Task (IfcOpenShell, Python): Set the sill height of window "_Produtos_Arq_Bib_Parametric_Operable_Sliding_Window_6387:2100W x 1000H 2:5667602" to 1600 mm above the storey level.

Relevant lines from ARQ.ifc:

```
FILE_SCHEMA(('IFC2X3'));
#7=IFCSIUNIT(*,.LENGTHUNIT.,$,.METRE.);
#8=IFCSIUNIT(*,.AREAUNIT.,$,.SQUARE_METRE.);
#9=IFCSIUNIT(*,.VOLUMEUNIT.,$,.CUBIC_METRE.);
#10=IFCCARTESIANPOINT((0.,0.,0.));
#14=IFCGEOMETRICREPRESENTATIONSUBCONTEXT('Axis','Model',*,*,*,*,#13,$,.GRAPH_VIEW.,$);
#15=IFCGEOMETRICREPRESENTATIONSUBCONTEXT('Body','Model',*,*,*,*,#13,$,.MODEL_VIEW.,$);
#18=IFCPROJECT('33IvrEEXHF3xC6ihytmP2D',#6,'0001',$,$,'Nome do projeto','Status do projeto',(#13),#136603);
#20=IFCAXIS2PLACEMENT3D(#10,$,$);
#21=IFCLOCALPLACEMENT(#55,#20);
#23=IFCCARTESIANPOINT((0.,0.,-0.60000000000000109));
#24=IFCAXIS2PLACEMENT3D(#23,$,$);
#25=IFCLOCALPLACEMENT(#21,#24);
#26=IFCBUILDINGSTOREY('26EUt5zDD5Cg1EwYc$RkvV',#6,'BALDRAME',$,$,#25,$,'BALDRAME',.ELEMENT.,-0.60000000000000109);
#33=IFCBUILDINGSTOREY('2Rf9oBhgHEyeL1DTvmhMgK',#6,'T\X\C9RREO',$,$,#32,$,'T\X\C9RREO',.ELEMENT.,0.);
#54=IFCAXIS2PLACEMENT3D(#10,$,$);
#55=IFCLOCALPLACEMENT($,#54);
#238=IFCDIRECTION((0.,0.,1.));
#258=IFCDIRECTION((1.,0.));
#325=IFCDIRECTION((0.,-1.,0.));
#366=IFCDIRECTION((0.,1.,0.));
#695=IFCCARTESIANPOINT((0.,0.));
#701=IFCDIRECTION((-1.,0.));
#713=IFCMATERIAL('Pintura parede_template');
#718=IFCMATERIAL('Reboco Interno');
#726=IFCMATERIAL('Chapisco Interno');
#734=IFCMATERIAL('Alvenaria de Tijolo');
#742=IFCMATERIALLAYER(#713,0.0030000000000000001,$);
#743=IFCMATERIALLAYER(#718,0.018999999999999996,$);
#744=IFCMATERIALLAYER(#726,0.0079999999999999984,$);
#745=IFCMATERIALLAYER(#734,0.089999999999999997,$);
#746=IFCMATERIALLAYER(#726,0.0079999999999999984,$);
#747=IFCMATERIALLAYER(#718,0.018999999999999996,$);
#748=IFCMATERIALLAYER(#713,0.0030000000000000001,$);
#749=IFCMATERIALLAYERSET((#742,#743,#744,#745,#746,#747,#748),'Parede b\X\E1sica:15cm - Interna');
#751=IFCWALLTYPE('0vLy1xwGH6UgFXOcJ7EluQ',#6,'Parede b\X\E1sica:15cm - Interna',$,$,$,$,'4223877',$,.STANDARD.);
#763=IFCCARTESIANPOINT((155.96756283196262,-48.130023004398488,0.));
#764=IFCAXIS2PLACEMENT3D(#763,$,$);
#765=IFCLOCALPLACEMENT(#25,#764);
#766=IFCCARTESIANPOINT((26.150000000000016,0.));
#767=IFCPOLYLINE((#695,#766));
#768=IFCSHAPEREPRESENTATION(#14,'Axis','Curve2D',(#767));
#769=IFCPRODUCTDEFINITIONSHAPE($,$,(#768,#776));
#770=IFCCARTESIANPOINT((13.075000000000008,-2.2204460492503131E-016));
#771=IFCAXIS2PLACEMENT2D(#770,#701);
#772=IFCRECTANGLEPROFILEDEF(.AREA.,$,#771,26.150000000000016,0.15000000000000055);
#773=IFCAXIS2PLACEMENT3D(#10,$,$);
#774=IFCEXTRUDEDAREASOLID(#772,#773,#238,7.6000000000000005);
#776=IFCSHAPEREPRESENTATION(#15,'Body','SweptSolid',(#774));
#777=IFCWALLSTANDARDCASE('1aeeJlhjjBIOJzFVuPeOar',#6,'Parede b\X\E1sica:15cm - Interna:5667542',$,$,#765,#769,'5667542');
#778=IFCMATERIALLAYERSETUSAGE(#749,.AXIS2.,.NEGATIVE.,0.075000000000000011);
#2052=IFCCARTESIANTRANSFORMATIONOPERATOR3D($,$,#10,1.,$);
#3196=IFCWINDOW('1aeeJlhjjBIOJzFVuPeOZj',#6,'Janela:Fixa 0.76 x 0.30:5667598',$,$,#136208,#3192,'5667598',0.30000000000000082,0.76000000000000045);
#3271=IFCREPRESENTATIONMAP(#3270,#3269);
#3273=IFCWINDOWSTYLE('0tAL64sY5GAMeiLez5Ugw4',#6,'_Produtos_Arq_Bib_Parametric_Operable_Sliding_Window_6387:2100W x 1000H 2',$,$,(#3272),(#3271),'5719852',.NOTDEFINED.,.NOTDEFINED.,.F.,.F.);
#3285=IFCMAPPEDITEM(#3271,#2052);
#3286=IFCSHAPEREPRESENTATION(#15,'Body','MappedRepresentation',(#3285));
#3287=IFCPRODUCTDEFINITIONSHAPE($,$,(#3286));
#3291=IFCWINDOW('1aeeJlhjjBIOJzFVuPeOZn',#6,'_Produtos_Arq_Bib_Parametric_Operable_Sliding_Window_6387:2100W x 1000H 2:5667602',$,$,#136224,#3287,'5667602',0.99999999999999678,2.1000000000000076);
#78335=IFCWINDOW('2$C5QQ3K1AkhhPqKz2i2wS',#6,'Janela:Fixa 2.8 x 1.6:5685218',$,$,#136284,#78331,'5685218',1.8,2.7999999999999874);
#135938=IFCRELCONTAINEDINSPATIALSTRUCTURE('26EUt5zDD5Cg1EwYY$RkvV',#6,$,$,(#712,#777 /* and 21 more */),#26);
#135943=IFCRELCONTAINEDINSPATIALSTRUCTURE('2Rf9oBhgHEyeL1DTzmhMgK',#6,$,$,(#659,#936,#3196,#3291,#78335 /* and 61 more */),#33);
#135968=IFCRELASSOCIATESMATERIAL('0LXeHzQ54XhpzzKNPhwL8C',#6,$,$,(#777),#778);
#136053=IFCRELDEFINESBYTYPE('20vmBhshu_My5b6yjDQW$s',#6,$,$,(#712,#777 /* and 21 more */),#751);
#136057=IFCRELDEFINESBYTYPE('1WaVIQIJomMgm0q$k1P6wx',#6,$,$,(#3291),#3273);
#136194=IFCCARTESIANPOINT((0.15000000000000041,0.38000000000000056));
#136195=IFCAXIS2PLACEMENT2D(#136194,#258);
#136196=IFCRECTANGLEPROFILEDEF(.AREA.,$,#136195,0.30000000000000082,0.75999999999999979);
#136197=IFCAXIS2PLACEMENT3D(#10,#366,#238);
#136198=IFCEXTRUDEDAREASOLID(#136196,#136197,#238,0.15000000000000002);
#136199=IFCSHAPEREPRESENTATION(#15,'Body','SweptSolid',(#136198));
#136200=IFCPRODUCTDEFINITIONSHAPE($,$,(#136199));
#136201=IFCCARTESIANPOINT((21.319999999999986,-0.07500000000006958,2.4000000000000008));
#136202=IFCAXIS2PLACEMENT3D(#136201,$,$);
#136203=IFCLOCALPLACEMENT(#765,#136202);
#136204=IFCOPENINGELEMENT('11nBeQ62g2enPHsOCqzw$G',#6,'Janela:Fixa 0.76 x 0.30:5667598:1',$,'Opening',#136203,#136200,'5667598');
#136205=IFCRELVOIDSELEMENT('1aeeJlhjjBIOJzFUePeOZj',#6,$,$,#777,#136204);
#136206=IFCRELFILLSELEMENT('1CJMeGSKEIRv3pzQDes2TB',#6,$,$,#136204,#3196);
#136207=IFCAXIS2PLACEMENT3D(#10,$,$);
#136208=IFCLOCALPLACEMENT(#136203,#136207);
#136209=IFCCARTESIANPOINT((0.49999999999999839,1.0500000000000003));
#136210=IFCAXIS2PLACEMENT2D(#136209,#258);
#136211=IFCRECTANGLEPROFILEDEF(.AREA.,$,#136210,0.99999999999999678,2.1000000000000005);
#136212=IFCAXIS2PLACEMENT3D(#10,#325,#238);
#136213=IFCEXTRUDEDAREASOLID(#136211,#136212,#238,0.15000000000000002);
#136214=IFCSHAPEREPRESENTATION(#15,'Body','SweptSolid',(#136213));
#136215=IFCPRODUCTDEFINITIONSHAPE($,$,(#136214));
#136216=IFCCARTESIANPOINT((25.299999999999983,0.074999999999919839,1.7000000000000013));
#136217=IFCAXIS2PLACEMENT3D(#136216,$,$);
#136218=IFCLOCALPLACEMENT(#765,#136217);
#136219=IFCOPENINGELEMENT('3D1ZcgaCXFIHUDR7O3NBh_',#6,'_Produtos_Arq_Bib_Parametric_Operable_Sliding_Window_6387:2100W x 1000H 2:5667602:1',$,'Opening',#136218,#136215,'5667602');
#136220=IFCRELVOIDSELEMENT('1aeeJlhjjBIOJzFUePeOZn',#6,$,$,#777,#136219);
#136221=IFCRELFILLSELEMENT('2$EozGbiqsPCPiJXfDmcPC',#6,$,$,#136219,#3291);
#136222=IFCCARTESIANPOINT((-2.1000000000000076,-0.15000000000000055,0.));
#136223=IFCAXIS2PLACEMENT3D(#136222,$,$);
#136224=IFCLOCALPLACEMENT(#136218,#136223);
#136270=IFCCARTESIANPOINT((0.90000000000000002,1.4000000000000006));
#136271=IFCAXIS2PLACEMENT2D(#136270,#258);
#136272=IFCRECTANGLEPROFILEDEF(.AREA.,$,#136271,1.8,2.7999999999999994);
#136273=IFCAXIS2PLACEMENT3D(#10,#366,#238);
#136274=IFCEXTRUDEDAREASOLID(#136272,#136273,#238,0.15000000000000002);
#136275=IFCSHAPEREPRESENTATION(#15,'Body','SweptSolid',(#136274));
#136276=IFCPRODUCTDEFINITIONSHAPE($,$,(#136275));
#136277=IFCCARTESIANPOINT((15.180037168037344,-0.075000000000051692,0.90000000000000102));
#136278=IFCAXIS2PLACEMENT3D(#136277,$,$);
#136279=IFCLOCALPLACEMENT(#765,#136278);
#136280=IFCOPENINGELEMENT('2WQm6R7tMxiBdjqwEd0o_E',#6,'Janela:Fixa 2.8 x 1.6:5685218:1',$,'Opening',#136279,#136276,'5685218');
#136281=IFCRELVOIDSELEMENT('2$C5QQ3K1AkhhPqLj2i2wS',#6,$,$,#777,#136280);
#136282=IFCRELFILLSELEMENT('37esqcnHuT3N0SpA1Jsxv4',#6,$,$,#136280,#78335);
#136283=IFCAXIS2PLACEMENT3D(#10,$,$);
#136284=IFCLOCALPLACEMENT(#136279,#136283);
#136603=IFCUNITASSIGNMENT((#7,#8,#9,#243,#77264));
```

```python
import numpy as np
import ifcopenshell
import ifcopenshell.api.geometry
import ifcopenshell.geom
import ifcopenshell.util.element
import ifcopenshell.util.placement
import ifcopenshell.util.shape
import ifcopenshell.util.unit

model = ifcopenshell.open("ARQ.ifc")
unit_scale = ifcopenshell.util.unit.calculate_unit_scale(model)

window = model.by_id(3291)
opening = window.FillsVoids[0].RelatingOpeningElement
storey = ifcopenshell.util.element.get_container(window, ifc_class="IfcBuildingStorey")
level = ifcopenshell.util.placement.get_local_placement(storey.ObjectPlacement)[2, 3]

# The opening's origin need not be at the sill, so measure its lowest point.
shape = ifcopenshell.geom.create_shape(ifcopenshell.geom.settings(), opening)
bottom = ifcopenshell.util.shape.get_shape_bottom_elevation(shape, shape.geometry) / unit_scale
dz = level + 1.6 - bottom

shift = np.array([0.0, 0.0, dz])
# The window is placed relative to its opening, so it follows when the opening moves.
matrix = ifcopenshell.util.placement.get_local_placement(opening.ObjectPlacement)
matrix[:3, 3] += shift
ifcopenshell.api.geometry.edit_object_placement(
    model, product=opening, matrix=matrix, is_si=False, should_transform_children=True
)

print(f"moved by {dz * unit_scale:+.3f} m")

model.write("ARQ_updated.ifc")
```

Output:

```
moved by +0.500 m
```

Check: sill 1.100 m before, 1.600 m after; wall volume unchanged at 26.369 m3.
